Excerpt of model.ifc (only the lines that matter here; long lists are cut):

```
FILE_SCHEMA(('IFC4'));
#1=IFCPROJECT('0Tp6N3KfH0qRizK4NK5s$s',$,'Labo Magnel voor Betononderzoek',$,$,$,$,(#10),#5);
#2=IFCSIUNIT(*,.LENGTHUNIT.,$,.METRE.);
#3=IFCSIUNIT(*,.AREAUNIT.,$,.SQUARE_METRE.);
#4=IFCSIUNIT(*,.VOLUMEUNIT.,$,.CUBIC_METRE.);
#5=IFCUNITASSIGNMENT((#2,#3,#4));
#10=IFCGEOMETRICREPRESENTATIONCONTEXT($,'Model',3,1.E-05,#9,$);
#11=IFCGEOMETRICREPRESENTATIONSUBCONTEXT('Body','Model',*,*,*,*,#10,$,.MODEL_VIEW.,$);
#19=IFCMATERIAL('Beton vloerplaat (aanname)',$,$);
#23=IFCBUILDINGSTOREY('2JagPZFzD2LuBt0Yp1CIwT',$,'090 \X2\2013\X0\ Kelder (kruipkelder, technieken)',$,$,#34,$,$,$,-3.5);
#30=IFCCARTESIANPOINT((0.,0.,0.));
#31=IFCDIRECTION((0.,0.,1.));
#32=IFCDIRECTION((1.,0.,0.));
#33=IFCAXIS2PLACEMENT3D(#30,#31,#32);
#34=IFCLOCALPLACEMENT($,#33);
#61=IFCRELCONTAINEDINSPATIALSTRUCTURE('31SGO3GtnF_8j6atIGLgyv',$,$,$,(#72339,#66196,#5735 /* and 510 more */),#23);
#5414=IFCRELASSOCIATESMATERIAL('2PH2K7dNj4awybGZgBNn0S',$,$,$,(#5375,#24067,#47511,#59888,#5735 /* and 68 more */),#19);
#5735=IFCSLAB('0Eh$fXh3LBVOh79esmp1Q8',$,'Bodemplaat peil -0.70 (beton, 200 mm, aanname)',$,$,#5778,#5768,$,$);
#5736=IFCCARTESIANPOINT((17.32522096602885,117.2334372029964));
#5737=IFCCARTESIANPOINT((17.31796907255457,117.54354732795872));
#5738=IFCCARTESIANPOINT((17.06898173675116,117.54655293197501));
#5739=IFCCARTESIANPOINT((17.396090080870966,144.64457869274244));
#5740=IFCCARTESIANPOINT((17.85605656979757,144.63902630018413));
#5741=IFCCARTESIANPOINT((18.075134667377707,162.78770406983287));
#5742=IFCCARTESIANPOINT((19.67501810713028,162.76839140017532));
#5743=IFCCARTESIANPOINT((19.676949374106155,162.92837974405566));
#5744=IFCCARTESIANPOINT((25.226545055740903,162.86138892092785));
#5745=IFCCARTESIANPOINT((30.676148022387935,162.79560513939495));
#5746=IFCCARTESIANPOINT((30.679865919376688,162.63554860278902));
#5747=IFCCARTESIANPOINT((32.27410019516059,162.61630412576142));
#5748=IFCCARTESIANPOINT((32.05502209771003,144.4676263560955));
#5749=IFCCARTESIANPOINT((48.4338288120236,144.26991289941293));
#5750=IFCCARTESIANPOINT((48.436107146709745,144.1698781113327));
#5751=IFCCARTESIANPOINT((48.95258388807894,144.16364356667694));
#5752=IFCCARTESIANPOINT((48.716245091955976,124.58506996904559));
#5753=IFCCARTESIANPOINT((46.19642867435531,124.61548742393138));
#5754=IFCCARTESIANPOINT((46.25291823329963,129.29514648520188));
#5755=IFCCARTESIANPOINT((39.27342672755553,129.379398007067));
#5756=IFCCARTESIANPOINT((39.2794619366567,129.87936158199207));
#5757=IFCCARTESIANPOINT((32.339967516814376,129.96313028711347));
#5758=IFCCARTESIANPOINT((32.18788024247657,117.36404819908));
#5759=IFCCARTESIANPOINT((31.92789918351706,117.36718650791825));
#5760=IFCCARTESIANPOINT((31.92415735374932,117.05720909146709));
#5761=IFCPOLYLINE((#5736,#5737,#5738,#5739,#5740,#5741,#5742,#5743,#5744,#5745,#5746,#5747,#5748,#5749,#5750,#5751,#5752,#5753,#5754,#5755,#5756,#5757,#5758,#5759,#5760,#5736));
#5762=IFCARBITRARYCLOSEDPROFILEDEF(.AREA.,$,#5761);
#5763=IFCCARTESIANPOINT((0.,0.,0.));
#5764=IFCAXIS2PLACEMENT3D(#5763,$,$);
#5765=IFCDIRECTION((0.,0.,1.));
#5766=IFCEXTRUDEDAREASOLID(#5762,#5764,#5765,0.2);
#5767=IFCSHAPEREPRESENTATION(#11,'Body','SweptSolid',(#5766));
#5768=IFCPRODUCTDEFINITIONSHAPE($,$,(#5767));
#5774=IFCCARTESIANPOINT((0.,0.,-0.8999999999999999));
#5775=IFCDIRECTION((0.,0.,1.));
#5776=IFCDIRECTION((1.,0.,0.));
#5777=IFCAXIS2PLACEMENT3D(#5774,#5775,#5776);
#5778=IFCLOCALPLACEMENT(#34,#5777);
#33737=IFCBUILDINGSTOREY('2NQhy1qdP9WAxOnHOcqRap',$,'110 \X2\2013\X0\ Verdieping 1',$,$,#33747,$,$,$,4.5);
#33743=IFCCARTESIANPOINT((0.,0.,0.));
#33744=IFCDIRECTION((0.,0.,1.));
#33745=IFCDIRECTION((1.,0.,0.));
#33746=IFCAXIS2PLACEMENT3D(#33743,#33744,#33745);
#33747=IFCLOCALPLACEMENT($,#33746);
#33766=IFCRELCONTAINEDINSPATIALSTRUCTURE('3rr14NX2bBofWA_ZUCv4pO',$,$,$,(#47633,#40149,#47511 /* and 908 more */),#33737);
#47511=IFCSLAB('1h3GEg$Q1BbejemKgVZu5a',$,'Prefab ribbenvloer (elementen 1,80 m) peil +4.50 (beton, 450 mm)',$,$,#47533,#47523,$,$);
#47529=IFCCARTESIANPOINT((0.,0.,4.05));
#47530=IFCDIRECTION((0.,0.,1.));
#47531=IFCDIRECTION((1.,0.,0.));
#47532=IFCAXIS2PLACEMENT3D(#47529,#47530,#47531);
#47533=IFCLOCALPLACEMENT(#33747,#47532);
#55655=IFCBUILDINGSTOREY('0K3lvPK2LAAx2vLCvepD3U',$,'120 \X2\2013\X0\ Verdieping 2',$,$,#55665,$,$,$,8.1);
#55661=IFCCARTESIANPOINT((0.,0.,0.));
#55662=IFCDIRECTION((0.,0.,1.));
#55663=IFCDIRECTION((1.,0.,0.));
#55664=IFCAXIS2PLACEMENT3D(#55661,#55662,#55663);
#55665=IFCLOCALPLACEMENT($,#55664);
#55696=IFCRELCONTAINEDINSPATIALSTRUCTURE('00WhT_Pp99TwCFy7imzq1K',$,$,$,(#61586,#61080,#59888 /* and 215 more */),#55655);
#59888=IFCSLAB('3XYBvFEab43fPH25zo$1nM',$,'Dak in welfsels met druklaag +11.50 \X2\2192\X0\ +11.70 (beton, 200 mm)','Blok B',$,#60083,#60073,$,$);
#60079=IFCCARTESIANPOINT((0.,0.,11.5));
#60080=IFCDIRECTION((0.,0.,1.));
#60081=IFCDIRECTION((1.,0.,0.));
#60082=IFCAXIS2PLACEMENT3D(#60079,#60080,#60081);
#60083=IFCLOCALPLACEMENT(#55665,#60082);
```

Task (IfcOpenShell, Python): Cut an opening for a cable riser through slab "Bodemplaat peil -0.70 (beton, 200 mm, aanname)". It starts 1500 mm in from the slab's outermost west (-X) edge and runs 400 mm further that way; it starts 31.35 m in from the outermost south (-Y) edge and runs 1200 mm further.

```python
import numpy as np
import ifcopenshell
import ifcopenshell.api.feature
import ifcopenshell.api.geometry
import ifcopenshell.api.root
import ifcopenshell.geom
import ifcopenshell.util.placement
import ifcopenshell.util.representation
import ifcopenshell.util.shape
import ifcopenshell.util.unit

model = ifcopenshell.open("model.ifc")
unit_scale = ifcopenshell.util.unit.calculate_unit_scale(model)
settings = ifcopenshell.geom.settings()


def volume(element):
    """Net volume in cubic metres, openings subtracted."""
    shape = ifcopenshell.geom.create_shape(settings, element)
    return ifcopenshell.util.shape.get_volume(shape.geometry)


slab = model.by_guid("0Eh$fXh3LBVOh79esmp1Q8")
before = volume(slab)

# Extent in the slab's own axes, in metres. The edges named are its -X and -Y sides.
slab_shape = ifcopenshell.geom.create_shape(settings, slab)
vertices = ifcopenshell.util.shape.get_vertices(slab_shape.geometry)
x_min, y_min, bottom = vertices.min(axis=0)
top = vertices[:, 2].max()

opening = ifcopenshell.api.root.create_entity(model, ifc_class="IfcOpeningElement", name="Cable riser opening", predefined_type="OPENING")
context = ifcopenshell.util.representation.get_context(model, "Model", "Body", "MODEL_VIEW")
width, depth = 0.4, 1.2
outline = [(0.0, 0.0), (width, 0.0), (width, depth), (0.0, depth), (0.0, 0.0)]
# Overshoot both faces by 50 mm so the cut is clean.
shape = ifcopenshell.api.geometry.add_slab_representation(
    model, context=context, depth=top - bottom + 0.1, polyline=outline
)
ifcopenshell.api.geometry.assign_representation(model, product=opening, representation=shape)

matrix = ifcopenshell.util.placement.get_local_placement(slab.ObjectPlacement)
matrix[:, 3] = matrix @ np.append(np.array([x_min + 1.5, y_min + 31.35, bottom - 0.05]) / unit_scale, 1.0)
ifcopenshell.api.geometry.edit_object_placement(model, product=opening, matrix=matrix, is_si=False)
ifcopenshell.api.feature.add_feature(model, feature=opening, element=slab)

after = volume(slab)

print(f"slab volume {before:.3f} -> {after:.3f} m3")

model.write("model_updated.ifc")
```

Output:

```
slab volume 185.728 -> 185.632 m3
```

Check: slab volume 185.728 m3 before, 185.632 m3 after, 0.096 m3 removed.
